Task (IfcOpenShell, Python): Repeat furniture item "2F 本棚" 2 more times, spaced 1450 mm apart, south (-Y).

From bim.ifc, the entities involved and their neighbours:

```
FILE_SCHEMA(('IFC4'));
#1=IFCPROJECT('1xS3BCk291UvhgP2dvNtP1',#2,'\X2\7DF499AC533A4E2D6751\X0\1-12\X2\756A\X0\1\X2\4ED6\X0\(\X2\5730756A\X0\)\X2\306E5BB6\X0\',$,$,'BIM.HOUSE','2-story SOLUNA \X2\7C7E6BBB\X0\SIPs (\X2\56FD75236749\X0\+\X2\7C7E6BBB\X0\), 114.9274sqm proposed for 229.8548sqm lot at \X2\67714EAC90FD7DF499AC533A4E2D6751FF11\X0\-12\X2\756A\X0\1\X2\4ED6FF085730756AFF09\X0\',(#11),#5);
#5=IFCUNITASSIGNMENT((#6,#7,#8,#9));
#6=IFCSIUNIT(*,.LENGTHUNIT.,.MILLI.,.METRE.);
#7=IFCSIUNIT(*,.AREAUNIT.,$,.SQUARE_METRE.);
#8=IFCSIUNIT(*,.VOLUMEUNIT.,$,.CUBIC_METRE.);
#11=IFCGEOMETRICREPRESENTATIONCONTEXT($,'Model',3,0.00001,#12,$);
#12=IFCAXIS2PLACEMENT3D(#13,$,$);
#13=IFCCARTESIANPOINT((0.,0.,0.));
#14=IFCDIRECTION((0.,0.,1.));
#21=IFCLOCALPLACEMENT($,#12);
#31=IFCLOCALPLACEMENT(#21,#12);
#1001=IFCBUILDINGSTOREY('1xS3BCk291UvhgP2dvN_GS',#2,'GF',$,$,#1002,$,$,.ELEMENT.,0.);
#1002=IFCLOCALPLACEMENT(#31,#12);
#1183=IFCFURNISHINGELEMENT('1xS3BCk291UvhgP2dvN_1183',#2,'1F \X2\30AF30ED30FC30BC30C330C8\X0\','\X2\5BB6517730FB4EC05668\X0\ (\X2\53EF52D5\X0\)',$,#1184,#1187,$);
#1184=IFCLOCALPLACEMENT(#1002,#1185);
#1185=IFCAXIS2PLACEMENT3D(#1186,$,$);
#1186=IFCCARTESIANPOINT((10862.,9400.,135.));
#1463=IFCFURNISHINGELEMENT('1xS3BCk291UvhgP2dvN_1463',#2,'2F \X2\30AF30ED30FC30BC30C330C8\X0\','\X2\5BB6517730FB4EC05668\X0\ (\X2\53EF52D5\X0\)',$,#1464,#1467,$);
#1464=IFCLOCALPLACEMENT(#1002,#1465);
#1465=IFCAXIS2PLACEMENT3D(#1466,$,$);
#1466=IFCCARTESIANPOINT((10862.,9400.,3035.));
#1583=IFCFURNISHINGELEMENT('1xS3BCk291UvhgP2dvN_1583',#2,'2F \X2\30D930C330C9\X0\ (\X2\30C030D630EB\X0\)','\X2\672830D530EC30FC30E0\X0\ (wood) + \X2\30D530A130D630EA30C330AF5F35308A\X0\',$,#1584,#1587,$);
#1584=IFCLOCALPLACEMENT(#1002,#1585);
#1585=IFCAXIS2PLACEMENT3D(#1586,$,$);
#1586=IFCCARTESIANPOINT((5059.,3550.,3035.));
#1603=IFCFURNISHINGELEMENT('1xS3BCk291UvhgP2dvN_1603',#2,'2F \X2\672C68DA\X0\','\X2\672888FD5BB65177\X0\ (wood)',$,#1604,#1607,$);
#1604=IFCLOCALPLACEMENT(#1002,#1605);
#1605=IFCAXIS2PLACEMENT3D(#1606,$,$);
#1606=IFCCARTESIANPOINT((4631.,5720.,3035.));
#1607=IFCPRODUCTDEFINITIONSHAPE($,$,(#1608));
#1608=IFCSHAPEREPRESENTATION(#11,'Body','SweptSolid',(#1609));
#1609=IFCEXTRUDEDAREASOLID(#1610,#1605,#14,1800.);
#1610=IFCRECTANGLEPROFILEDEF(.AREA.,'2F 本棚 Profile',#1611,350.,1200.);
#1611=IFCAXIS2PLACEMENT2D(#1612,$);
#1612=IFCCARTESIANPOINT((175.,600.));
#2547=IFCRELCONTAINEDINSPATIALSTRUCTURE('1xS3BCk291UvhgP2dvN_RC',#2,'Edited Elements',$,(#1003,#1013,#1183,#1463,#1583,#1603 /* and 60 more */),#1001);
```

```python
import numpy as np
import ifcopenshell
import ifcopenshell.api.geometry
import ifcopenshell.api.root
import ifcopenshell.util.element
import ifcopenshell.util.placement
import ifcopenshell.util.unit

model = ifcopenshell.open("bim.ifc")
unit_scale = ifcopenshell.util.unit.calculate_unit_scale(model)


def reuse_history(source, copy):
    """copy_class also copies each property set's owner history, people and application; keep the originals."""
    for rel in copy.IsDefinedBy:
        if rel.is_a("IfcRelDefinesByProperties") and (history := rel.RelatingPropertyDefinition.OwnerHistory):
            rel.RelatingPropertyDefinition.OwnerHistory = source.OwnerHistory
            ifcopenshell.util.element.remove_deep2(model, history)


source = model.by_id(1603)
base = ifcopenshell.util.placement.get_local_placement(source.ObjectPlacement)
step = np.array([0.0, -1.0, 0.0]) * 1.45 / unit_scale

for i in range(1, 3):
    copy = ifcopenshell.api.root.copy_class(model, product=source)
    copy.Representation = ifcopenshell.util.element.copy_deep(
        model, source.Representation, exclude=["IfcGeometricRepresentationContext", "IfcRepresentationMap"]
    )
    reuse_history(source, copy)
    matrix = base.copy()
    matrix[:3, 3] += i * step
    print("added at", matrix[:3, 3].round(3) + 0.0)
    ifcopenshell.api.geometry.edit_object_placement(model, product=copy, matrix=matrix, is_si=False)

model.write("bim-out.ifc")
```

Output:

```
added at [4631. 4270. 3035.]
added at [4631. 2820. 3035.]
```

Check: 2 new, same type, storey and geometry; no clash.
